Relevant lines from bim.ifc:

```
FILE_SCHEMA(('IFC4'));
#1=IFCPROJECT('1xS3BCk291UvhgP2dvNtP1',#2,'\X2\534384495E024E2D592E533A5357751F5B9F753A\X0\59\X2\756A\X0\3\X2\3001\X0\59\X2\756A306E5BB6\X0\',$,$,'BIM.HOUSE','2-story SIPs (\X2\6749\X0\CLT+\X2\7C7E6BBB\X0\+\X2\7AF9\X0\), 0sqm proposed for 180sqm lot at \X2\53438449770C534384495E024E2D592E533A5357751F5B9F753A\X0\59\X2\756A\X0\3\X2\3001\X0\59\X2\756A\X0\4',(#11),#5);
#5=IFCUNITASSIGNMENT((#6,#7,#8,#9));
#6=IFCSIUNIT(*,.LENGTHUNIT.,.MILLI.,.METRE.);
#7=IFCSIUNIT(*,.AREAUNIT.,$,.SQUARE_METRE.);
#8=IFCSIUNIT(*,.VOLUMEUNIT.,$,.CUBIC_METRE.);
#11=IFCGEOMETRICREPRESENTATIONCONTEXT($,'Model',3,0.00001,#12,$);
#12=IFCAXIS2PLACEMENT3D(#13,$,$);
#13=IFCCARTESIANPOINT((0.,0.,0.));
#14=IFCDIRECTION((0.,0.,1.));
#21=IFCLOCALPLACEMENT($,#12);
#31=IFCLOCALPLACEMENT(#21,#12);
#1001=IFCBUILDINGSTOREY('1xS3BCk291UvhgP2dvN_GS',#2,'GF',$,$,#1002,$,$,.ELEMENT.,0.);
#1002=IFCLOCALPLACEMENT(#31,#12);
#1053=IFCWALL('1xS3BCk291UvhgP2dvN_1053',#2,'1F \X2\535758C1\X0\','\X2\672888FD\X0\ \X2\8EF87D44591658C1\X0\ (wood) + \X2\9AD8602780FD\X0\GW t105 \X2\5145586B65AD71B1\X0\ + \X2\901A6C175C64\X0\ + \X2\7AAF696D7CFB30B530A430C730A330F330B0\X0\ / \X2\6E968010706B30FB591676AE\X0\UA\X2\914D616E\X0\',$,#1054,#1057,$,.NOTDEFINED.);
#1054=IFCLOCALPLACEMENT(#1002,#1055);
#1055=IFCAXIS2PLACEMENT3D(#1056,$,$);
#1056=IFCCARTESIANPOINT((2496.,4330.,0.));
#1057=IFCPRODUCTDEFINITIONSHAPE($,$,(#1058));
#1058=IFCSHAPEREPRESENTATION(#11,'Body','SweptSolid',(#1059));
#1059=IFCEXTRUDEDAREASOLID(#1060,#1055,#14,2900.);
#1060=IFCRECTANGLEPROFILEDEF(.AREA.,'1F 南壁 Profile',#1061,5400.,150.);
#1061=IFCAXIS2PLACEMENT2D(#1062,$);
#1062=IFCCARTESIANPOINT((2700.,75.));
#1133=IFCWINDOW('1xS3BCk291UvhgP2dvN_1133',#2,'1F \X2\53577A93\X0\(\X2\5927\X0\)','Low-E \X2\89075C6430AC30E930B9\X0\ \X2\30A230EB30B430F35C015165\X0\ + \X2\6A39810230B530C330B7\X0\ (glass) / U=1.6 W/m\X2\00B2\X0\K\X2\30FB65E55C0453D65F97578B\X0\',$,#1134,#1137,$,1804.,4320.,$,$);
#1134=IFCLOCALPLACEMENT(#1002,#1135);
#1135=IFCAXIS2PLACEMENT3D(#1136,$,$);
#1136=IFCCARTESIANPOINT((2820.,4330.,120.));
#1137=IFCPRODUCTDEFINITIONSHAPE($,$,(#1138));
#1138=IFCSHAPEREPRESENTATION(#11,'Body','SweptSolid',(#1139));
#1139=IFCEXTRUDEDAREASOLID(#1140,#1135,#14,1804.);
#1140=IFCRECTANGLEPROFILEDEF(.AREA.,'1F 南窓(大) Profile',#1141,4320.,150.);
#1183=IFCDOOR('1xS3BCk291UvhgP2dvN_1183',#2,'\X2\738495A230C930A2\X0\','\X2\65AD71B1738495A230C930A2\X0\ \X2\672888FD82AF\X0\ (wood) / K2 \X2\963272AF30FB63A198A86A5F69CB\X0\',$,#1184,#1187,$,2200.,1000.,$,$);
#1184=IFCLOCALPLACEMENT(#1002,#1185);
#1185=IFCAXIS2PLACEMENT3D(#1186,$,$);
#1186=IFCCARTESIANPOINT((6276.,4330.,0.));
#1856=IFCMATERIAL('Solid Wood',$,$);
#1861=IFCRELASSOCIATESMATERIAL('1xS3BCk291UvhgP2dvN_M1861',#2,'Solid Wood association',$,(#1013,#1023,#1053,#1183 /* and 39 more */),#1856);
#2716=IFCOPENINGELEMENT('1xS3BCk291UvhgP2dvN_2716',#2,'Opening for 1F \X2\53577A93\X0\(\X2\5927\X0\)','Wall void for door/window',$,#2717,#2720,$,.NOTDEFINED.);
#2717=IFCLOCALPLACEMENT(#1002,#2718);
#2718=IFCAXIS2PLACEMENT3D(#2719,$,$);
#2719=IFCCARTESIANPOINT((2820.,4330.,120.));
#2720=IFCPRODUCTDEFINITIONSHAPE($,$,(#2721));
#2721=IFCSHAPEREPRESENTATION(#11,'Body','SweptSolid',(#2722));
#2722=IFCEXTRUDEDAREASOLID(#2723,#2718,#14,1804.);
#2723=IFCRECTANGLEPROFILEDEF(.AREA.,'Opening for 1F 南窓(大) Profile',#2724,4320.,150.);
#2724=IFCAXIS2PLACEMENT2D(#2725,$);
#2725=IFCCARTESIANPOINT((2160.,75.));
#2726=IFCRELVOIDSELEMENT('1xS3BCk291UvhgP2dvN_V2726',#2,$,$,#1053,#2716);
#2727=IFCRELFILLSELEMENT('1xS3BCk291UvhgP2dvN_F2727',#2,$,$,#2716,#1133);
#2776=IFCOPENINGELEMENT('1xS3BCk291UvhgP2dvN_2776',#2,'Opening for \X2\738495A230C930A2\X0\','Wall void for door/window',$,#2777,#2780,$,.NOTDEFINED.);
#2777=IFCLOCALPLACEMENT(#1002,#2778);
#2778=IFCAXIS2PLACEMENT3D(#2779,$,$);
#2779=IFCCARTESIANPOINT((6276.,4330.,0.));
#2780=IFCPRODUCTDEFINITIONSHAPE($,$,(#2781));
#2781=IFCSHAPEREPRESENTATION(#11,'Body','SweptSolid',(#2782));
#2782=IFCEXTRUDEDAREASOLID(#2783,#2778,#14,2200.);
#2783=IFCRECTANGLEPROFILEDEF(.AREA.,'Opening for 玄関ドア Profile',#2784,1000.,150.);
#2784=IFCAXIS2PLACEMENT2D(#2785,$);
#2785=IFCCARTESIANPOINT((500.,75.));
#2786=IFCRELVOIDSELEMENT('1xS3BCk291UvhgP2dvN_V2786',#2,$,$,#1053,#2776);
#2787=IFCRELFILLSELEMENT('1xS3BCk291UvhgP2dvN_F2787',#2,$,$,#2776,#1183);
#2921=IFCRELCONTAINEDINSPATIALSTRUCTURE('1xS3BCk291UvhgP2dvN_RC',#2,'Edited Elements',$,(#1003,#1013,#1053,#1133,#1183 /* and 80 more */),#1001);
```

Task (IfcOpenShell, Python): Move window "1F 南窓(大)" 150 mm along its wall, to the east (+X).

```python
import ifcopenshell
import ifcopenshell.api.geometry
import ifcopenshell.util.placement

model = ifcopenshell.open("bim.ifc")

window = model.by_guid("1xS3BCk291UvhgP2dvN_1133")
opening = window.FillsVoids[0].RelatingOpeningElement
wall = opening.VoidsElements[0].RelatingBuildingElement

wall_matrix = ifcopenshell.util.placement.get_local_placement(wall.ObjectPlacement)
shift = wall_matrix[:3, 0] * 150.0
before = ifcopenshell.util.placement.get_local_placement(window.ObjectPlacement)[:3, 3].copy()

# The window is not placed relative to its opening, so move both.
for product in (opening, window):
    matrix = ifcopenshell.util.placement.get_local_placement(product.ObjectPlacement)
    matrix[:3, 3] += shift
    ifcopenshell.api.geometry.edit_object_placement(model, product=product, matrix=matrix, is_si=False)

after = ifcopenshell.util.placement.get_local_placement(window.ObjectPlacement)[:3, 3]
print("window moved by", (after - before).round(3) + 0.0)

model.write("bim_rev.ifc")
```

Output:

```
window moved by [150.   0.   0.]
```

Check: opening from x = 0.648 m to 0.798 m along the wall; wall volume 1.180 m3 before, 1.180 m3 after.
